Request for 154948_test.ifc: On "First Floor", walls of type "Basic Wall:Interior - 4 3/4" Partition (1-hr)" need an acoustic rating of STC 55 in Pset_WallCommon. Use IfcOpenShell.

First a look at what the model holds.

```python
import ifcopenshell
import ifcopenshell.util.element

model = ifcopenshell.open("154948_test.ifc")
print(model.schema)
storey = next(s for s in model.by_type("IfcBuildingStorey") if s.Name == "First Floor")
walls = [e for e in ifcopenshell.util.element.get_decomposition(storey) if e.is_a("IfcWall")]
seen = {}
for e in walls:
    element_type = ifcopenshell.util.element.get_type(e)
    key = (element_type.Name if element_type != e and element_type else None, ifcopenshell.util.element.get_pset(e, "Pset_WallCommon", "AcousticRating"))
    seen[key] = seen.get(key, 0) + 1
for (name, value), count in sorted(seen.items(), key=str):
    print(count, "x", name, "|", value)
```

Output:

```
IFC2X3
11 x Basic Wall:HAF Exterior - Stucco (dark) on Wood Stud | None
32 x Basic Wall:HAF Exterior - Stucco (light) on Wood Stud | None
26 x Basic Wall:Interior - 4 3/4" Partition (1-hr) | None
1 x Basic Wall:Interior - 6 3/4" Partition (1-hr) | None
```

```python
import ifcopenshell
import ifcopenshell.api.pset
import ifcopenshell.util.element

model = ifcopenshell.open("154948_test.ifc")

storey = next(s for s in model.by_type("IfcBuildingStorey") if s.Name == "First Floor")
walls = [e for e in ifcopenshell.util.element.get_decomposition(storey) if e.is_a("IfcWall")]

count = 0
for e in walls:
    element_type = ifcopenshell.util.element.get_type(e)
    if element_type in (None, e) or element_type.Name != 'Basic Wall:Interior - 4 3/4" Partition (1-hr)':
        continue
    # add_pset returns the element's existing set when there is one.
    pset = ifcopenshell.api.pset.add_pset(model, product=e, name="Pset_WallCommon")
    ifcopenshell.api.pset.edit_pset(model, pset=pset, properties={"AcousticRating": "STC 55"})
    count += 1

print(count, "walls updated")

model.write("154948_test_rev.ifc")
```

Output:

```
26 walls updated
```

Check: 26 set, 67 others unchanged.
